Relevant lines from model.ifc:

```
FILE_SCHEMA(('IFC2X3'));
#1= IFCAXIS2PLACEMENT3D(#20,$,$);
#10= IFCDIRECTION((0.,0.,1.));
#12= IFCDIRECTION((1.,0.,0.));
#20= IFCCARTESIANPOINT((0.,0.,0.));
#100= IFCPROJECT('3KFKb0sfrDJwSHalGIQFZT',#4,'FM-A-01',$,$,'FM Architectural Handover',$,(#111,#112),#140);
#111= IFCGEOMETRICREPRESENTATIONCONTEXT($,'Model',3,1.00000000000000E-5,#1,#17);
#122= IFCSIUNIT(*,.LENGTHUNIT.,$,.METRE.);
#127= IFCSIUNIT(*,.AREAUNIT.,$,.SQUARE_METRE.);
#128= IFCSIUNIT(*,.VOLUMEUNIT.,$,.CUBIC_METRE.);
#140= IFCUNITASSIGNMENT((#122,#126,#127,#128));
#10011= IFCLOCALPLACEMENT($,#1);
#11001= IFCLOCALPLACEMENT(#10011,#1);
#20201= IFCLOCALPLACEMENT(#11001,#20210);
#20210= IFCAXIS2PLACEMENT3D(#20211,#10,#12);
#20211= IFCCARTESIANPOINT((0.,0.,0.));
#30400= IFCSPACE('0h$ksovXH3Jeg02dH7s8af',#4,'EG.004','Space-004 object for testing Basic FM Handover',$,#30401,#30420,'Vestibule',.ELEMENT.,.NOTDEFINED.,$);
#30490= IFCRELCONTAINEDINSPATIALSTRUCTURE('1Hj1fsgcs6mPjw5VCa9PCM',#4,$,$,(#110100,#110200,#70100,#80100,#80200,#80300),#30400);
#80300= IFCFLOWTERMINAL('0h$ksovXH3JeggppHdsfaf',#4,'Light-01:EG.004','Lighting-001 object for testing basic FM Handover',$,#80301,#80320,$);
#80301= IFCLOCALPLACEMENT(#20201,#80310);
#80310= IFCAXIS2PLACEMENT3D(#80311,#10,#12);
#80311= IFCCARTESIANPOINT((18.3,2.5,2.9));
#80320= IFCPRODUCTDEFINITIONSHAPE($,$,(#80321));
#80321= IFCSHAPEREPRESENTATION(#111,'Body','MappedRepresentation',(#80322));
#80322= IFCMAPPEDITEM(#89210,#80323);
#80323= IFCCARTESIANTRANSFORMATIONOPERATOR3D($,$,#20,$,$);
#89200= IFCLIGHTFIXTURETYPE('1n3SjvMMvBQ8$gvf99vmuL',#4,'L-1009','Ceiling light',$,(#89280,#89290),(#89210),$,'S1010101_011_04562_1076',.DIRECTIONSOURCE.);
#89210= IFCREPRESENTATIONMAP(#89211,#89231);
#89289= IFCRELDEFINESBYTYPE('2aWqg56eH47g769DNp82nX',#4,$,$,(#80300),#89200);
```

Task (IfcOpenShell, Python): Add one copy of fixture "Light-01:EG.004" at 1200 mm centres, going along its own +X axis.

```python
import ifcopenshell
import ifcopenshell.api.geometry
import ifcopenshell.api.root
import ifcopenshell.util.element
import ifcopenshell.util.placement

model = ifcopenshell.open("model.ifc")

source = model.by_guid("0h$ksovXH3JeggppHdsfaf")
base = ifcopenshell.util.placement.get_local_placement(source.ObjectPlacement)
step = base[:3, 0] * 1.2

for i in range(1, 2):
    copy = ifcopenshell.api.root.copy_class(model, product=source)
    copy.Representation = ifcopenshell.util.element.copy_deep(
        model, source.Representation, exclude=["IfcGeometricRepresentationContext", "IfcRepresentationMap"]
    )
    matrix = base.copy()
    matrix[:3, 3] += i * step
    print("added at", matrix[:3, 3].round(3) + 0.0)
    ifcopenshell.api.geometry.edit_object_placement(model, product=copy, matrix=matrix, is_si=False)

model.write("model-out.ifc")
```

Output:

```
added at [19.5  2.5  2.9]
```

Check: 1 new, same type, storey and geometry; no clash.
